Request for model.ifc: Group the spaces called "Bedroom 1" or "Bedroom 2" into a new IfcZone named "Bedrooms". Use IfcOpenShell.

First a look at what the model holds.

```python
import ifcopenshell

model = ifcopenshell.open("model.ifc")
print(model.schema)
seen = {}
for space in model.by_type("IfcSpace"):
    seen[space.LongName] = seen.get(space.LongName, 0) + 1
for name, count in sorted(seen.items(), key=str):
    print(count, "x", name)
print("zones:", [z.Name for z in model.by_type("IfcZone")][:20])
```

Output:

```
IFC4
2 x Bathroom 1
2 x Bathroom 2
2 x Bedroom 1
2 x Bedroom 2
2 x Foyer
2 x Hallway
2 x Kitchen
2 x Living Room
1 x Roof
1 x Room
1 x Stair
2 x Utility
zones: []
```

```python
import ifcopenshell
import ifcopenshell.api.group
import ifcopenshell.api.root

model = ifcopenshell.open("model.ifc")

names = {"Bedroom 1", "Bedroom 2"}
spaces = [s for s in model.by_type("IfcSpace") if s.LongName in names]

zone = ifcopenshell.api.root.create_entity(model, ifc_class="IfcZone", name="Bedrooms")
ifcopenshell.api.group.assign_group(model, products=spaces, group=zone)
print(len(spaces), "spaces in", zone.Name)

model.write("model_rev.ifc")
```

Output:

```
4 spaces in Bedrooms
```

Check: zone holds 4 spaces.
